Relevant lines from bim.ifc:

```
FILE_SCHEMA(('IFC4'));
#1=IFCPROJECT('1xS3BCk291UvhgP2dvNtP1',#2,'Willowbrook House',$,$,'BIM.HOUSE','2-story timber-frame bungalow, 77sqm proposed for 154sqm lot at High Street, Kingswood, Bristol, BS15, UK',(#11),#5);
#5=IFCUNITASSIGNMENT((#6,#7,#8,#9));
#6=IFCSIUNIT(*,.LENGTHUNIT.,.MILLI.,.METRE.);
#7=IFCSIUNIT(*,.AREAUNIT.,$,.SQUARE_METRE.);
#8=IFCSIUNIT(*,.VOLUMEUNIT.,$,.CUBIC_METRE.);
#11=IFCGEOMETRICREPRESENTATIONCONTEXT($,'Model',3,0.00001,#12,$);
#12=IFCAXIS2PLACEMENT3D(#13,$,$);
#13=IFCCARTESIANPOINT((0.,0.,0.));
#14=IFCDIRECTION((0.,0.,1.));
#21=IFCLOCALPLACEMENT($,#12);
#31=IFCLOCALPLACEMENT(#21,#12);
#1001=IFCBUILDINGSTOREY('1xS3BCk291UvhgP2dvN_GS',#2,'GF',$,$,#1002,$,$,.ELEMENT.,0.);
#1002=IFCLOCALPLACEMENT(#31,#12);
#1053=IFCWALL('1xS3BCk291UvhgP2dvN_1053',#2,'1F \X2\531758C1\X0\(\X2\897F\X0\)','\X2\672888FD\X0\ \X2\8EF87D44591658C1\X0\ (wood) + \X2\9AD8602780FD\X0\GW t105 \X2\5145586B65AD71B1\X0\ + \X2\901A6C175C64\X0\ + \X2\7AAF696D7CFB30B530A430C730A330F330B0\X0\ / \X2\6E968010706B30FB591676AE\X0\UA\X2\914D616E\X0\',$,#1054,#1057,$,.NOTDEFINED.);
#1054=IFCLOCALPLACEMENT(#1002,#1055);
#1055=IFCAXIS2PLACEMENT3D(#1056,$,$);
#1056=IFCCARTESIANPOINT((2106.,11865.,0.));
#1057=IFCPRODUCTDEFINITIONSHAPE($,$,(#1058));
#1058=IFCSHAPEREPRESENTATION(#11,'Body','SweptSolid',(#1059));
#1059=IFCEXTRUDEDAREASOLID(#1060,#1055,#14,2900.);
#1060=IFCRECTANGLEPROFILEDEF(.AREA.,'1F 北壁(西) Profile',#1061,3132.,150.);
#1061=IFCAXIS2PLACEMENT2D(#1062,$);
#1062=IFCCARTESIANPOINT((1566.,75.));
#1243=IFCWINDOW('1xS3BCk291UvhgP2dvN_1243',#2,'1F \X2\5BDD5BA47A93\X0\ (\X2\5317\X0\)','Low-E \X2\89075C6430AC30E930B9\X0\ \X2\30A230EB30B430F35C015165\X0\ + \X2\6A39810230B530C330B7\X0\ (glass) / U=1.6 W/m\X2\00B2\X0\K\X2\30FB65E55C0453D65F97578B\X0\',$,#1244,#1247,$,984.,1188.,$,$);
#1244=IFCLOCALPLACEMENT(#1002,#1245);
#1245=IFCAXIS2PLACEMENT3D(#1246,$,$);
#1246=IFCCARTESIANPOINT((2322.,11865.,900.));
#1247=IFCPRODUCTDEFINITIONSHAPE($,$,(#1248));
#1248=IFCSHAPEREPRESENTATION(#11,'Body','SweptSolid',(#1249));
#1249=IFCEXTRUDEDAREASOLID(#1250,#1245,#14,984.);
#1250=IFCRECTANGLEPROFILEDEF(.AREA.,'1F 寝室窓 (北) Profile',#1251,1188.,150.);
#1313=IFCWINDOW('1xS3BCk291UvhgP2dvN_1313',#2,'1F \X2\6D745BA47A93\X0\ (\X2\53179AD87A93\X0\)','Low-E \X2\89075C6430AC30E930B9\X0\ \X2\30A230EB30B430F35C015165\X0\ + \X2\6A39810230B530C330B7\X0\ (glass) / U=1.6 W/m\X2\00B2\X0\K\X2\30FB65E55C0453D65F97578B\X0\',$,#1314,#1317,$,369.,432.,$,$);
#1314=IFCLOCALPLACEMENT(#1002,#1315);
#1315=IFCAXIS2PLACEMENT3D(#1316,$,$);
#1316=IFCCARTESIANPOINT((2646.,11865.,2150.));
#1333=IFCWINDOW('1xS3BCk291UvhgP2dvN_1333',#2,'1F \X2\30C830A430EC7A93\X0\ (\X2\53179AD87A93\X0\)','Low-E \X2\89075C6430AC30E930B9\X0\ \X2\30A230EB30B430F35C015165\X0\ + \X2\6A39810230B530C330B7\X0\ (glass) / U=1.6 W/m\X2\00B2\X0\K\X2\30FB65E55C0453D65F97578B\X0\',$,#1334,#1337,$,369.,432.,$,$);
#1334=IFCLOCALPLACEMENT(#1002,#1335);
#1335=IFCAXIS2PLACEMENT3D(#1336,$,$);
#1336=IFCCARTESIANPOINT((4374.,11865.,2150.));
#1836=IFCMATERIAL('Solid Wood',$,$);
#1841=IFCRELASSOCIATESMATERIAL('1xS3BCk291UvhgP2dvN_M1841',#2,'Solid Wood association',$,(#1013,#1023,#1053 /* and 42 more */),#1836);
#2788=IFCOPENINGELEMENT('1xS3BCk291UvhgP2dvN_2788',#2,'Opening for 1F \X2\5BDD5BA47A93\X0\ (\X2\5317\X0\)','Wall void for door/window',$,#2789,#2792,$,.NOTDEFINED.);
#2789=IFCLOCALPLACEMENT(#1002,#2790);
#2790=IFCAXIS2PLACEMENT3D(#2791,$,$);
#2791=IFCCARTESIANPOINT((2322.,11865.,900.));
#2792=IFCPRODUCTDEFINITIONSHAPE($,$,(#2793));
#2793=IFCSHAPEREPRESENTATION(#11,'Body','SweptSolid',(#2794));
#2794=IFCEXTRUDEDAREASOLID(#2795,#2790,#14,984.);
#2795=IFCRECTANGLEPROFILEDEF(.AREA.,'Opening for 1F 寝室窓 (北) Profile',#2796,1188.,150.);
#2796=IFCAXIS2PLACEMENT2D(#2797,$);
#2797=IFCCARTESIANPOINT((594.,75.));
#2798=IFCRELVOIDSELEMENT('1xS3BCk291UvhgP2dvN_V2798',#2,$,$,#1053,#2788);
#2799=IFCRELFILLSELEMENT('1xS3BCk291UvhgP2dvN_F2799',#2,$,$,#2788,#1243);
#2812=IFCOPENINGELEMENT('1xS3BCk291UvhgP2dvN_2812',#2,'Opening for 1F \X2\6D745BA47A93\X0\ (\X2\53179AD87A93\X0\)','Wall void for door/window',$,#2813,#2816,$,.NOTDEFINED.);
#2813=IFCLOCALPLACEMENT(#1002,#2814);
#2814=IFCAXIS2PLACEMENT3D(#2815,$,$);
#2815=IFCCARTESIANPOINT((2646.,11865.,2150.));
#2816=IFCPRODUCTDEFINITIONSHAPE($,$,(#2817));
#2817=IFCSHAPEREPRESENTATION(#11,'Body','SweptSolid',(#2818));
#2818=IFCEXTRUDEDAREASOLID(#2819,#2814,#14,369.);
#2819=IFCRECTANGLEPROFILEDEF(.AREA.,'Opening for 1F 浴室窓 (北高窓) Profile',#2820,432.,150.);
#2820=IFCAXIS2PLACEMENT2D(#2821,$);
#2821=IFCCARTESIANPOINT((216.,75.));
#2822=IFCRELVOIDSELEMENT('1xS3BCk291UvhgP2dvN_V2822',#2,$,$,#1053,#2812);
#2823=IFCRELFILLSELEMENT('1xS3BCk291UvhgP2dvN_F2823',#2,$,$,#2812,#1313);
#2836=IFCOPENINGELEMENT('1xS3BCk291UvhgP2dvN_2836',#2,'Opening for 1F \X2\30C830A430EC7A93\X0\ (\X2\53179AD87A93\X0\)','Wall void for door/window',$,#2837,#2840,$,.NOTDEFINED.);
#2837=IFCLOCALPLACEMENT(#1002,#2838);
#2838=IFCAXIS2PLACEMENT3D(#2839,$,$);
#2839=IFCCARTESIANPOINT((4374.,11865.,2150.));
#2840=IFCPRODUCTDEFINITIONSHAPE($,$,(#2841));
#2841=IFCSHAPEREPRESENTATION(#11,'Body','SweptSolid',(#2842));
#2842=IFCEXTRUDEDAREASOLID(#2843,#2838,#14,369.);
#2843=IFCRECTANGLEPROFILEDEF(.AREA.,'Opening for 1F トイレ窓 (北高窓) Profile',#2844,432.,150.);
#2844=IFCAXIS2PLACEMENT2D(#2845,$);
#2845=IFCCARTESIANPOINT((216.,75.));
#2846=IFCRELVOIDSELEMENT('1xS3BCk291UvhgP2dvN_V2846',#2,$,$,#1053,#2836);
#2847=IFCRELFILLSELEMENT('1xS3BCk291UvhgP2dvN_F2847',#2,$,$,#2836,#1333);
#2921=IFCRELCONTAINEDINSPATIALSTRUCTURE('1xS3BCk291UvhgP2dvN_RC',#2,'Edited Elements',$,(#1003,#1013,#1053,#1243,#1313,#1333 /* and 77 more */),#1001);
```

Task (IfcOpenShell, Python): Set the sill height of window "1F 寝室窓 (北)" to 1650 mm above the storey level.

```python
import numpy as np
import ifcopenshell
import ifcopenshell.api.geometry
import ifcopenshell.geom
import ifcopenshell.util.element
import ifcopenshell.util.placement
import ifcopenshell.util.shape
import ifcopenshell.util.unit

model = ifcopenshell.open("bim.ifc")
unit_scale = ifcopenshell.util.unit.calculate_unit_scale(model)

window = model.by_guid("1xS3BCk291UvhgP2dvN_1243")
opening = window.FillsVoids[0].RelatingOpeningElement
storey = ifcopenshell.util.element.get_container(window, ifc_class="IfcBuildingStorey")
level = ifcopenshell.util.placement.get_local_placement(storey.ObjectPlacement)[2, 3]

# The opening's origin need not be at the sill, so measure its lowest point.
shape = ifcopenshell.geom.create_shape(ifcopenshell.geom.settings(), opening)
bottom = ifcopenshell.util.shape.get_shape_bottom_elevation(shape, shape.geometry) / unit_scale
dz = level + 1.65 / unit_scale - bottom

shift = np.array([0.0, 0.0, dz])
# The window is not placed relative to its opening, so move both.
for product in (opening, window):
    matrix = ifcopenshell.util.placement.get_local_placement(product.ObjectPlacement)
    matrix[:3, 3] += shift
    ifcopenshell.api.geometry.edit_object_placement(model, product=product, matrix=matrix, is_si=False)

print(f"moved by {dz * unit_scale:+.3f} m")

model.write("bim_v2.ifc")
```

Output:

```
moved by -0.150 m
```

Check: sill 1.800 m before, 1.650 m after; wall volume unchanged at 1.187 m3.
